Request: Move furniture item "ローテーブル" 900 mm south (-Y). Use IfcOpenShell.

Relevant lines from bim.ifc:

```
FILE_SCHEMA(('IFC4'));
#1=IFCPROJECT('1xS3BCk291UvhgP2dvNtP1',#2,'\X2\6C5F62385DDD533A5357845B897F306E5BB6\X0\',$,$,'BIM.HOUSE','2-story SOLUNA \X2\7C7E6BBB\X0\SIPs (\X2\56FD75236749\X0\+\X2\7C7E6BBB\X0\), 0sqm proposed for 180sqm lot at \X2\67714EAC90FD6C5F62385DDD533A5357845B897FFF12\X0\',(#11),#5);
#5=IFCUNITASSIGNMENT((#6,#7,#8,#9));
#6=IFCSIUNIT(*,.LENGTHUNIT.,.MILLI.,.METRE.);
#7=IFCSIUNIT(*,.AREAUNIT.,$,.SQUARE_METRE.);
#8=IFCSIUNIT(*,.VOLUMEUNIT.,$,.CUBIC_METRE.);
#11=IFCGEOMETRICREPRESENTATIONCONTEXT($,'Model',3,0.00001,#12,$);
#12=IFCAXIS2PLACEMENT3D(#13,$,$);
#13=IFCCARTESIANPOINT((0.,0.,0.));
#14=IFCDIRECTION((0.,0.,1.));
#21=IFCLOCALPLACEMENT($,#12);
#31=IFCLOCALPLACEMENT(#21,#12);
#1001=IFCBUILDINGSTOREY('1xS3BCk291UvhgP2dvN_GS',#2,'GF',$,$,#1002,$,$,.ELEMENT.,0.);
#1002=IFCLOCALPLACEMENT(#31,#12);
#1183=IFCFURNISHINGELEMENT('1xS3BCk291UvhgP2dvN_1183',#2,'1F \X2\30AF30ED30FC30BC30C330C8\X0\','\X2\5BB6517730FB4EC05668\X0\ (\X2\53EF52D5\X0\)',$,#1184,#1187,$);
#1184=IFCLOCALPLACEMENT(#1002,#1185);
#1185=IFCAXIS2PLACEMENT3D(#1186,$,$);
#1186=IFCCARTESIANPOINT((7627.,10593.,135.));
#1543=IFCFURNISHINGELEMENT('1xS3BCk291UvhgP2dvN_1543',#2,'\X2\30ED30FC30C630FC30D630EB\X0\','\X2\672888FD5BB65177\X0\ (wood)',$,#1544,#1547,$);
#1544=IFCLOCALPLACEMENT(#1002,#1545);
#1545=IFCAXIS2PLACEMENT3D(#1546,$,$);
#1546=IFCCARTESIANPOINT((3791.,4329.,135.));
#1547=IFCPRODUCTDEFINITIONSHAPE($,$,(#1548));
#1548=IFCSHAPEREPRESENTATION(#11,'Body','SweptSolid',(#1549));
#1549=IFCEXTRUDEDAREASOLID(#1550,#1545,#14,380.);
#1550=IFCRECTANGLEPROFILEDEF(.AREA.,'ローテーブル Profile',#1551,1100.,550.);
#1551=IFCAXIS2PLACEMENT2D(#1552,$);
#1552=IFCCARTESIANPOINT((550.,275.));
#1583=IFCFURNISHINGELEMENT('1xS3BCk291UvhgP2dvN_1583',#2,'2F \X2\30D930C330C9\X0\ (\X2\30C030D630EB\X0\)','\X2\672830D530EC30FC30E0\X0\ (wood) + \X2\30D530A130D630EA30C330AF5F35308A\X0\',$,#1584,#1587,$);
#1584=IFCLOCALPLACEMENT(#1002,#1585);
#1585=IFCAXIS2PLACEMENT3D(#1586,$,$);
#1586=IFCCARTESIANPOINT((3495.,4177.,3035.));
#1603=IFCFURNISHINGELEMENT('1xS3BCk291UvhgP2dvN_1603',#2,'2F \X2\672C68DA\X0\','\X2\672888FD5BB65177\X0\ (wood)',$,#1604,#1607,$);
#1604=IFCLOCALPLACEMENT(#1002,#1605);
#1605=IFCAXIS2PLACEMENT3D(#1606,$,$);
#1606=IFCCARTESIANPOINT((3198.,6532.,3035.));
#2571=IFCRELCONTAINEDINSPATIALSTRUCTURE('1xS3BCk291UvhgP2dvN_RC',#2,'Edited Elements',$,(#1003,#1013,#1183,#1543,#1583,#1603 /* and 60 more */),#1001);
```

```python
import ifcopenshell
import ifcopenshell.api.geometry
import ifcopenshell.util.placement
import ifcopenshell.util.unit

model = ifcopenshell.open("bim.ifc")
unit_scale = ifcopenshell.util.unit.calculate_unit_scale(model)

item = model.by_id(1543)
matrix = ifcopenshell.util.placement.get_local_placement(item.ObjectPlacement)
matrix[1, 3] -= 0.9 / unit_scale
ifcopenshell.api.geometry.edit_object_placement(model, product=item, matrix=matrix, is_si=False)

print(ifcopenshell.util.placement.get_local_placement(item.ObjectPlacement).round(3) + 0.0)

model.write("bim_edited.ifc")
```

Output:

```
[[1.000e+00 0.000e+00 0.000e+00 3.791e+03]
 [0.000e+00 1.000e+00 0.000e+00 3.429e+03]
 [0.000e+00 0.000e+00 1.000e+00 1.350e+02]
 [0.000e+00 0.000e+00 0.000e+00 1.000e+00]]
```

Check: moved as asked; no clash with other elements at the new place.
